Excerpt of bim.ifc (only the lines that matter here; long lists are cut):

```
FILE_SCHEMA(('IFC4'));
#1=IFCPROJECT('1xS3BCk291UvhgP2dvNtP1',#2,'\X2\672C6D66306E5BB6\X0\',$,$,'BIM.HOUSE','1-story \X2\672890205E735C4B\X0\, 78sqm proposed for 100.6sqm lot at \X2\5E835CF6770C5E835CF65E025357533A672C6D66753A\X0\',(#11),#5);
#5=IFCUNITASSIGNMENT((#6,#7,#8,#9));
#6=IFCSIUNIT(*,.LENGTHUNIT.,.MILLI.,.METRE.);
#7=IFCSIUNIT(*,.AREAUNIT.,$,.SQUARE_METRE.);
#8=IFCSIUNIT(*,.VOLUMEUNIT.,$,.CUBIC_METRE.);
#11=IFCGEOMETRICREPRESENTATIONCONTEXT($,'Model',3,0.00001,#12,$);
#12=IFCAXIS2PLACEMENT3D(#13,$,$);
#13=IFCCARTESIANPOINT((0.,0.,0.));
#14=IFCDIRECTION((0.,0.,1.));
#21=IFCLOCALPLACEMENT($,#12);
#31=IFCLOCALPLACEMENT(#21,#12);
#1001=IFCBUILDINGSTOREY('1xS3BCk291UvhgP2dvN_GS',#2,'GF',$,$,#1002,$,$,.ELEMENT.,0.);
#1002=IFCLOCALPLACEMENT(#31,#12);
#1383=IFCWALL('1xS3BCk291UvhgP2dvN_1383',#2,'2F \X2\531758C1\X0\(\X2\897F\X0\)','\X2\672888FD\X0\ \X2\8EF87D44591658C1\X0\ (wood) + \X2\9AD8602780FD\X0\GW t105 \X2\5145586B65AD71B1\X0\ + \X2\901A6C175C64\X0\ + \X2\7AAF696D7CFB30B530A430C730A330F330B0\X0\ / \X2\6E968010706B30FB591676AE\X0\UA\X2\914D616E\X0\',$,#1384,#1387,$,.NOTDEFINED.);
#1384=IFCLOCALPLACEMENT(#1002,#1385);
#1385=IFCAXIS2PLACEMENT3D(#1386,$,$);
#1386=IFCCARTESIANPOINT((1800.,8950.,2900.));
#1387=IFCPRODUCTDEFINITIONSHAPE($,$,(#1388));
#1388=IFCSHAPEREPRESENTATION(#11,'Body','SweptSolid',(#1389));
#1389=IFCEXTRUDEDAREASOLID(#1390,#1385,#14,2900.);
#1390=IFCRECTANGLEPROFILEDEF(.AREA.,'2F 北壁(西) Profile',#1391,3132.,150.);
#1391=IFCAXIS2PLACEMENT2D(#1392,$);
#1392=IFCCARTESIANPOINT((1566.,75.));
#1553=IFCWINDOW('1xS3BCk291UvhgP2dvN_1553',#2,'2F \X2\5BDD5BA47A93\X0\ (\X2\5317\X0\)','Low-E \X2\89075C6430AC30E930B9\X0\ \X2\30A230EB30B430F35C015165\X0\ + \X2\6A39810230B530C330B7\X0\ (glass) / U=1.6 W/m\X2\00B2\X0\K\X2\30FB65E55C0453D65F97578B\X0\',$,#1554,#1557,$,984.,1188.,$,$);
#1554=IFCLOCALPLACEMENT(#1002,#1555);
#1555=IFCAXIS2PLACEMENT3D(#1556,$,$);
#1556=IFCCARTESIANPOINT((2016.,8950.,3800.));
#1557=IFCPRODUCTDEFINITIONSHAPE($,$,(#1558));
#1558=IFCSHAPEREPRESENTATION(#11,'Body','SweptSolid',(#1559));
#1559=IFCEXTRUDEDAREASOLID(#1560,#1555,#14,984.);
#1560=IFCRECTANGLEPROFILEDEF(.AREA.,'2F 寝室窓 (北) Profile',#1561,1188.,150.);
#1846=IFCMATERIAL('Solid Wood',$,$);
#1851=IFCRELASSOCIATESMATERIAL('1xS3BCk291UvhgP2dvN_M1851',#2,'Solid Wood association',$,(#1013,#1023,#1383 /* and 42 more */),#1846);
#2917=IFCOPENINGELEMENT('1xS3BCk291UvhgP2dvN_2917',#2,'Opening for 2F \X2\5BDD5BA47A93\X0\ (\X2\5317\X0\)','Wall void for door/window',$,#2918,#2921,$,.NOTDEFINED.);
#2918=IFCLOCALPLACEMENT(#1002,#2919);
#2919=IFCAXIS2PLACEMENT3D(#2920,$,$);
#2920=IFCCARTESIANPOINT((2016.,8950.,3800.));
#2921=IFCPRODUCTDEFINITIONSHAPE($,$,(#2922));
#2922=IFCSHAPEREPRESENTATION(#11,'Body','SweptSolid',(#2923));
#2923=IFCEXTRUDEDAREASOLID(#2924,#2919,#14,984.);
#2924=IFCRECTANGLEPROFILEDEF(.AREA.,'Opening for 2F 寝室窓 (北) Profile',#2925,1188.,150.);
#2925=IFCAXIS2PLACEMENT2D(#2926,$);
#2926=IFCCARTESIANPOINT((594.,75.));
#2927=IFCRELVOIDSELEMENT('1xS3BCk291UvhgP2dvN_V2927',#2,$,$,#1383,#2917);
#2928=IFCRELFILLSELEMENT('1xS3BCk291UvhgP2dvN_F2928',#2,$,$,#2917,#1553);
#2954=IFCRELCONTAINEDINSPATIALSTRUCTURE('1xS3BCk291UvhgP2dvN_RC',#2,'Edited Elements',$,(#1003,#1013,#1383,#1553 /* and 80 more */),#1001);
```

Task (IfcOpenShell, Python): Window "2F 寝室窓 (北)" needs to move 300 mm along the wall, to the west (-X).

```python
import ifcopenshell
import ifcopenshell.api.geometry
import ifcopenshell.util.placement
import ifcopenshell.util.unit

model = ifcopenshell.open("bim.ifc")
unit_scale = ifcopenshell.util.unit.calculate_unit_scale(model)

window = model.by_id(1553)
opening = window.FillsVoids[0].RelatingOpeningElement
wall = opening.VoidsElements[0].RelatingBuildingElement

wall_matrix = ifcopenshell.util.placement.get_local_placement(wall.ObjectPlacement)
shift = wall_matrix[:3, 0] * -0.3 / unit_scale
before = ifcopenshell.util.placement.get_local_placement(window.ObjectPlacement)[:3, 3].copy()

# The window is not placed relative to its opening, so move both.
for product in (opening, window):
    matrix = ifcopenshell.util.placement.get_local_placement(product.ObjectPlacement)
    matrix[:3, 3] += shift
    ifcopenshell.api.geometry.edit_object_placement(model, product=product, matrix=matrix, is_si=False)

after = ifcopenshell.util.placement.get_local_placement(window.ObjectPlacement)[:3, 3]
print("window moved by", (after - before).round(3) + 0.0)

model.write("bim_edited.ifc")
```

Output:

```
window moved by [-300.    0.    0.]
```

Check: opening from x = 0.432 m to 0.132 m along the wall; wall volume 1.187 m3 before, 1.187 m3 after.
